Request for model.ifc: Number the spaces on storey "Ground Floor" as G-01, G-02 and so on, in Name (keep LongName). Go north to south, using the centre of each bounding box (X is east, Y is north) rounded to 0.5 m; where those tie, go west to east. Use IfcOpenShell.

First a look at what the model holds.

```python
import ifcopenshell
import ifcopenshell.util.element
import ifcopenshell.util.placement

model = ifcopenshell.open("model.ifc")
print(model.schema)
storey = next(s for s in model.by_type("IfcBuildingStorey") if s.Name == "Ground Floor")
spaces = [e for e in ifcopenshell.util.element.get_decomposition(storey) if e.is_a("IfcSpace")]
for e in sorted(spaces, key=lambda e: e.id()):
    origin = ifcopenshell.util.placement.get_local_placement(e.ObjectPlacement)[:3, 3]
    print(e.id(), e.Name, e.LongName, origin.round(2) + 0.0, sep=" | ")
```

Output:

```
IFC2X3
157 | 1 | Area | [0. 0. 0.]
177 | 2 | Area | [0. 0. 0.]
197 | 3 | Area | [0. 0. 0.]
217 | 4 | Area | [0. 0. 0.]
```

```python
import ifcopenshell
import ifcopenshell.geom
import ifcopenshell.util.element
import ifcopenshell.util.shape

model = ifcopenshell.open("model.ifc")
settings = ifcopenshell.geom.settings()
settings.set("use-world-coords", True)


def centre(element):
    shape = ifcopenshell.geom.create_shape(settings, element)
    return ifcopenshell.util.shape.get_bbox_centroid(shape.geometry)


storey = next(s for s in model.by_type("IfcBuildingStorey") if s.Name == "Ground Floor")
spaces = [e for e in ifcopenshell.util.element.get_decomposition(storey) if e.is_a("IfcSpace")]

# Insertion points can sit at a corner or the storey origin, so sort by the geometry (in metres).
centres = {e: centre(e) for e in spaces}
spaces.sort(key=lambda e: (-round(centres[e][1] / 0.5), centres[e][0]))

for i, e in enumerate(spaces, start=1):
    number = f"G-{i:02d}"
    e.Name = number
    print(e.id(), number)

model.write("model-out.ifc")
```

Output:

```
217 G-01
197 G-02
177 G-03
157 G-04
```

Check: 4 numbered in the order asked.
